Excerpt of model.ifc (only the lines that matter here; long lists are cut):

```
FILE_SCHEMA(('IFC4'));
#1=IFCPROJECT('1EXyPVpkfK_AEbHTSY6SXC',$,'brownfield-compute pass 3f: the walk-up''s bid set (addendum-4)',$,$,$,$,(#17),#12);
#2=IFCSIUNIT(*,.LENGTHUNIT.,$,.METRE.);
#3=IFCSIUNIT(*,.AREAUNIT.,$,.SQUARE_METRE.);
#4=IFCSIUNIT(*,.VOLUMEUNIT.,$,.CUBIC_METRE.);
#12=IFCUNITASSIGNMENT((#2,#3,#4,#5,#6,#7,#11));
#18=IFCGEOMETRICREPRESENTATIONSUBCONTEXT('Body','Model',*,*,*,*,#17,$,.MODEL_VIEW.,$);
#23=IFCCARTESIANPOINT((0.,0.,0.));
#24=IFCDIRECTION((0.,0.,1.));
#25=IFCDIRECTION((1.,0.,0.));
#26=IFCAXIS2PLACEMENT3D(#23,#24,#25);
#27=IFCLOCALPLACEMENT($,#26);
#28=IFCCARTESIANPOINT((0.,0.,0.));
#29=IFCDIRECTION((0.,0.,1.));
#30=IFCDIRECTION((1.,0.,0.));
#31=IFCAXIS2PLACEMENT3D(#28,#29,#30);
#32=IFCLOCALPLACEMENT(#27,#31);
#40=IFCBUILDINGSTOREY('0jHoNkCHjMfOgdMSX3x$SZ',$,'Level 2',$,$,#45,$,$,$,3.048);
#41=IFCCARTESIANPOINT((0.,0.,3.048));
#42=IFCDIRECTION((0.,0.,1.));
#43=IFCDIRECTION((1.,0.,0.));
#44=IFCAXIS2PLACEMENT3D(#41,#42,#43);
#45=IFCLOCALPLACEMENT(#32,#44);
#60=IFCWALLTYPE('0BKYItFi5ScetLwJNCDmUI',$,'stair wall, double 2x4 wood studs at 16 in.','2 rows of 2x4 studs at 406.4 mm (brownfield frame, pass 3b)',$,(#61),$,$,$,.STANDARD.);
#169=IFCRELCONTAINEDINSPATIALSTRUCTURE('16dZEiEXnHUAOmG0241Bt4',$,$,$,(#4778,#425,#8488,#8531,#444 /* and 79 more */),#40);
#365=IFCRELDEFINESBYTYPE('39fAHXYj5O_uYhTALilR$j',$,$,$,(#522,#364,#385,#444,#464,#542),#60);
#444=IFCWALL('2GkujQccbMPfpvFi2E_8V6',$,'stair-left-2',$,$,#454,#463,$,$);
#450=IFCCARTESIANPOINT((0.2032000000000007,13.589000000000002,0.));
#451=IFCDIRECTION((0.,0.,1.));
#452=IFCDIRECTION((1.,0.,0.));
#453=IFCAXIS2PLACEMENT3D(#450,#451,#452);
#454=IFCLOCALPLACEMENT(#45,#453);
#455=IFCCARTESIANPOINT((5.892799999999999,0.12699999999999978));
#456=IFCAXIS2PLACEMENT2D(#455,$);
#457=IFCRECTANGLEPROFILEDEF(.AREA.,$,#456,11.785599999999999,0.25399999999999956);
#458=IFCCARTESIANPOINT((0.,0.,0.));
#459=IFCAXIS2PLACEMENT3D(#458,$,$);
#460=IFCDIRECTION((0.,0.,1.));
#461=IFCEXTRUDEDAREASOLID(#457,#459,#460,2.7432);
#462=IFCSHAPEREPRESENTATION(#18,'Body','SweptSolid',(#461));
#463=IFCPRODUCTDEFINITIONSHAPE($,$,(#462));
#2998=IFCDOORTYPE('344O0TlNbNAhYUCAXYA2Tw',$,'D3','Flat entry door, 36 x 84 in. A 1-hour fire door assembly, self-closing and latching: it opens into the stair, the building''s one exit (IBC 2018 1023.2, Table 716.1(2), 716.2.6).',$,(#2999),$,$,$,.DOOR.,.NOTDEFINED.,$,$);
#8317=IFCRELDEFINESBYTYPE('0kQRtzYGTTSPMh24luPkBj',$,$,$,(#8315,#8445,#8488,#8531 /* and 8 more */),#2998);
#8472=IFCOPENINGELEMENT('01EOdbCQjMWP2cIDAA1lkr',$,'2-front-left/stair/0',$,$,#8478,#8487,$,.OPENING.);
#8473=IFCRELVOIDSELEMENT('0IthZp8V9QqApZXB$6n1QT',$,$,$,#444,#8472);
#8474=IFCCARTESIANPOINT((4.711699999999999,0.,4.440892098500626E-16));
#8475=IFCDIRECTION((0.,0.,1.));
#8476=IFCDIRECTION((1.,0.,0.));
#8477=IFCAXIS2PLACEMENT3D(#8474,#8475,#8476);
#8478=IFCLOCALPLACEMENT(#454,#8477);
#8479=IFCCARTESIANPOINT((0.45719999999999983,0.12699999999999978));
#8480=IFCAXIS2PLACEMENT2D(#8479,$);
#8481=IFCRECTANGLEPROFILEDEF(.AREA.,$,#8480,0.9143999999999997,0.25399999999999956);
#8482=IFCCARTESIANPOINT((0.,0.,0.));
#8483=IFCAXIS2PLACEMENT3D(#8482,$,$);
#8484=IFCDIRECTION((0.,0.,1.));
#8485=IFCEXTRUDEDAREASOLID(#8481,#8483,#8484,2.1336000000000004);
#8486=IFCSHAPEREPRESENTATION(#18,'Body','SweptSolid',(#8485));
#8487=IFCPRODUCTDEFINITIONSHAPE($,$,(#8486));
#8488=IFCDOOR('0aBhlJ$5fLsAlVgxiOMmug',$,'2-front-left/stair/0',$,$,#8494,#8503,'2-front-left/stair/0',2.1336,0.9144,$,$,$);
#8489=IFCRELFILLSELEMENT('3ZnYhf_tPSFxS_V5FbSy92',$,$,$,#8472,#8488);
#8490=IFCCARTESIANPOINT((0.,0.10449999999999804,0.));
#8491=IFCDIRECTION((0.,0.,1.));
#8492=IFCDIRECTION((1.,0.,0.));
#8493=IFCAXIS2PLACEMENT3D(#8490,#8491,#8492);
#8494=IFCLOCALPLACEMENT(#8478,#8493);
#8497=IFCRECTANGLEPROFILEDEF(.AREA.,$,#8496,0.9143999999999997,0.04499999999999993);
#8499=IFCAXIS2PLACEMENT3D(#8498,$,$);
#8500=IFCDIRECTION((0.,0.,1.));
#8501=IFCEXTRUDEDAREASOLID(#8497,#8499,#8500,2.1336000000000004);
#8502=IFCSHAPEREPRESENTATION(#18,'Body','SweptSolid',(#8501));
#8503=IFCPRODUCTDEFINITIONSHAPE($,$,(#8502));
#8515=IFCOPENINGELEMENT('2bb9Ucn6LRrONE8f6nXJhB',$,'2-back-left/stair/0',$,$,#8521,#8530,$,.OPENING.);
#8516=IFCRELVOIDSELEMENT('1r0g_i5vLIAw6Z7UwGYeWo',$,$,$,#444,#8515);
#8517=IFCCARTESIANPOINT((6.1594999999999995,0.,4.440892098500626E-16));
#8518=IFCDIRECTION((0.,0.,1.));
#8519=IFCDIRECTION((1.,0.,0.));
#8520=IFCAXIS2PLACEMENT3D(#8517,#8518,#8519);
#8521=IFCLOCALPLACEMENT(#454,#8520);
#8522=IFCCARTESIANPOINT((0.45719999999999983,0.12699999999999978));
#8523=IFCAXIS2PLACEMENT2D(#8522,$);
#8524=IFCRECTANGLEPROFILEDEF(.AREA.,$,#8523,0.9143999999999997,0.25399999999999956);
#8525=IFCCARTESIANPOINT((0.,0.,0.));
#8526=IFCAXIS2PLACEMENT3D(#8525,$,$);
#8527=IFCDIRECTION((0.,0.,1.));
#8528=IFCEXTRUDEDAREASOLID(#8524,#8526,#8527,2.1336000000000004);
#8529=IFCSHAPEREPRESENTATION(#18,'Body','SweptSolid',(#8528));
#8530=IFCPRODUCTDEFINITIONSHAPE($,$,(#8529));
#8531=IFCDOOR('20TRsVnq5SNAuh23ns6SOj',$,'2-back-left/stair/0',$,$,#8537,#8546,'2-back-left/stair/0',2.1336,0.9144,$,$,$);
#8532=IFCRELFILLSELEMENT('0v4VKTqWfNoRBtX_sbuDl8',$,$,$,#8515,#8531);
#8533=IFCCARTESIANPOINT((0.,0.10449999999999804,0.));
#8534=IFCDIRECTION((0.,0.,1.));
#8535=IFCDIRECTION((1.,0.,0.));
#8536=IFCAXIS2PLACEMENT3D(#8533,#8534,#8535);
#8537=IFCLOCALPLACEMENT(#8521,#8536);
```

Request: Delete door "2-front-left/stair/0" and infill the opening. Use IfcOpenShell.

```python
import ifcopenshell
import ifcopenshell.api.feature
import ifcopenshell.api.root
import ifcopenshell.geom
import ifcopenshell.util.shape

model = ifcopenshell.open("model.ifc")
settings = ifcopenshell.geom.settings()


def volume(element):
    """Net volume in cubic metres, openings subtracted."""
    shape = ifcopenshell.geom.create_shape(settings, element)
    return ifcopenshell.util.shape.get_volume(shape.geometry)


door = model.by_guid("0aBhlJ$5fLsAlVgxiOMmug")
opening = door.FillsVoids[0].RelatingOpeningElement
wall = opening.VoidsElements[0].RelatingBuildingElement
before = volume(wall)

ifcopenshell.api.root.remove_product(model, product=door)
ifcopenshell.api.feature.remove_feature(model, feature=opening)

after = volume(wall)

print(f"wall volume {before:.3f} -> {after:.3f} m3")

model.write("model_v2.ifc")
```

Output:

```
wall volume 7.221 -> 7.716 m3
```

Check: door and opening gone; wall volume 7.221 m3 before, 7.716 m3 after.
